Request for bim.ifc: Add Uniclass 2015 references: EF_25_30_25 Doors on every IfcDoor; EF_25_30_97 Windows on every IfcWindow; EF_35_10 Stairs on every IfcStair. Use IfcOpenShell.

First a look at what the model holds.

```python
import ifcopenshell

model = ifcopenshell.open("bim.ifc")
print(model.schema)
print("classifications:", [c.Name for c in model.by_type("IfcClassification")])
for ifc_class in ("IfcDoor", "IfcRoof", "IfcStair", "IfcWall", "IfcWindow"):
    print(ifc_class, len(model.by_type(ifc_class)))
```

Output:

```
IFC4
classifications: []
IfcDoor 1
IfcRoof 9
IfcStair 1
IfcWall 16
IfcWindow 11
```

```python
import ifcopenshell
import ifcopenshell.api.classification

model = ifcopenshell.open("bim.ifc")

system = ifcopenshell.api.classification.add_classification(model, classification="Uniclass 2015")

codes = {
    "IfcDoor": ("EF_25_30_25", "Doors"),
    "IfcWindow": ("EF_25_30_97", "Windows"),
    "IfcStair": ("EF_35_10", "Stairs"),
}
for ifc_class, (code, name) in codes.items():
    products = model.by_type(ifc_class)
    ifcopenshell.api.classification.add_reference(
        model, products=products, classification=system, identification=code, name=name
    )
    print(code, len(products))

model.write("bim_edited.ifc")
```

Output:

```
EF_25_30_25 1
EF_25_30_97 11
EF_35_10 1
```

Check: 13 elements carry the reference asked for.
